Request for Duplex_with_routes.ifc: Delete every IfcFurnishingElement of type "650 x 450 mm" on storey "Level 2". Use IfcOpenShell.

First a look at what the model holds.

```python
import ifcopenshell
import ifcopenshell.util.element

model = ifcopenshell.open("Duplex_with_routes.ifc")
print(model.schema)
storey = next(s for s in model.by_type("IfcBuildingStorey") if s.Name == "Level 2")
furniture = [e for e in ifcopenshell.util.element.get_decomposition(storey) if e.is_a("IfcFurnishingElement")]
seen = {}
for e in furniture:
    element_type = ifcopenshell.util.element.get_type(e)
    name = element_type.Name if element_type not in (None, e) else None
    seen[name] = seen.get(name, 0) + 1
for name, count in sorted(seen.items(), key=str):
    print(count, "x", name)
```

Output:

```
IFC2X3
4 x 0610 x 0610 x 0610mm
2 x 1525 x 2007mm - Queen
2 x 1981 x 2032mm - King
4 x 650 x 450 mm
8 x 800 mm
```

```python
import ifcopenshell
import ifcopenshell.api.root
import ifcopenshell.util.element

model = ifcopenshell.open("Duplex_with_routes.ifc")

storey = next(s for s in model.by_type("IfcBuildingStorey") if s.Name == "Level 2")
furniture = [e for e in ifcopenshell.util.element.get_decomposition(storey) if e.is_a("IfcFurnishingElement")]
targets = [e for e in furniture if (t := ifcopenshell.util.element.get_type(e)) not in (None, e) and t.Name == "650 x 450 mm"]

for e in targets:
    ifcopenshell.api.root.remove_product(model, product=e)
print(len(targets), "removed")

model.write("Duplex_with_routes_v2.ifc")
```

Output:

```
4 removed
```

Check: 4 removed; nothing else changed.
